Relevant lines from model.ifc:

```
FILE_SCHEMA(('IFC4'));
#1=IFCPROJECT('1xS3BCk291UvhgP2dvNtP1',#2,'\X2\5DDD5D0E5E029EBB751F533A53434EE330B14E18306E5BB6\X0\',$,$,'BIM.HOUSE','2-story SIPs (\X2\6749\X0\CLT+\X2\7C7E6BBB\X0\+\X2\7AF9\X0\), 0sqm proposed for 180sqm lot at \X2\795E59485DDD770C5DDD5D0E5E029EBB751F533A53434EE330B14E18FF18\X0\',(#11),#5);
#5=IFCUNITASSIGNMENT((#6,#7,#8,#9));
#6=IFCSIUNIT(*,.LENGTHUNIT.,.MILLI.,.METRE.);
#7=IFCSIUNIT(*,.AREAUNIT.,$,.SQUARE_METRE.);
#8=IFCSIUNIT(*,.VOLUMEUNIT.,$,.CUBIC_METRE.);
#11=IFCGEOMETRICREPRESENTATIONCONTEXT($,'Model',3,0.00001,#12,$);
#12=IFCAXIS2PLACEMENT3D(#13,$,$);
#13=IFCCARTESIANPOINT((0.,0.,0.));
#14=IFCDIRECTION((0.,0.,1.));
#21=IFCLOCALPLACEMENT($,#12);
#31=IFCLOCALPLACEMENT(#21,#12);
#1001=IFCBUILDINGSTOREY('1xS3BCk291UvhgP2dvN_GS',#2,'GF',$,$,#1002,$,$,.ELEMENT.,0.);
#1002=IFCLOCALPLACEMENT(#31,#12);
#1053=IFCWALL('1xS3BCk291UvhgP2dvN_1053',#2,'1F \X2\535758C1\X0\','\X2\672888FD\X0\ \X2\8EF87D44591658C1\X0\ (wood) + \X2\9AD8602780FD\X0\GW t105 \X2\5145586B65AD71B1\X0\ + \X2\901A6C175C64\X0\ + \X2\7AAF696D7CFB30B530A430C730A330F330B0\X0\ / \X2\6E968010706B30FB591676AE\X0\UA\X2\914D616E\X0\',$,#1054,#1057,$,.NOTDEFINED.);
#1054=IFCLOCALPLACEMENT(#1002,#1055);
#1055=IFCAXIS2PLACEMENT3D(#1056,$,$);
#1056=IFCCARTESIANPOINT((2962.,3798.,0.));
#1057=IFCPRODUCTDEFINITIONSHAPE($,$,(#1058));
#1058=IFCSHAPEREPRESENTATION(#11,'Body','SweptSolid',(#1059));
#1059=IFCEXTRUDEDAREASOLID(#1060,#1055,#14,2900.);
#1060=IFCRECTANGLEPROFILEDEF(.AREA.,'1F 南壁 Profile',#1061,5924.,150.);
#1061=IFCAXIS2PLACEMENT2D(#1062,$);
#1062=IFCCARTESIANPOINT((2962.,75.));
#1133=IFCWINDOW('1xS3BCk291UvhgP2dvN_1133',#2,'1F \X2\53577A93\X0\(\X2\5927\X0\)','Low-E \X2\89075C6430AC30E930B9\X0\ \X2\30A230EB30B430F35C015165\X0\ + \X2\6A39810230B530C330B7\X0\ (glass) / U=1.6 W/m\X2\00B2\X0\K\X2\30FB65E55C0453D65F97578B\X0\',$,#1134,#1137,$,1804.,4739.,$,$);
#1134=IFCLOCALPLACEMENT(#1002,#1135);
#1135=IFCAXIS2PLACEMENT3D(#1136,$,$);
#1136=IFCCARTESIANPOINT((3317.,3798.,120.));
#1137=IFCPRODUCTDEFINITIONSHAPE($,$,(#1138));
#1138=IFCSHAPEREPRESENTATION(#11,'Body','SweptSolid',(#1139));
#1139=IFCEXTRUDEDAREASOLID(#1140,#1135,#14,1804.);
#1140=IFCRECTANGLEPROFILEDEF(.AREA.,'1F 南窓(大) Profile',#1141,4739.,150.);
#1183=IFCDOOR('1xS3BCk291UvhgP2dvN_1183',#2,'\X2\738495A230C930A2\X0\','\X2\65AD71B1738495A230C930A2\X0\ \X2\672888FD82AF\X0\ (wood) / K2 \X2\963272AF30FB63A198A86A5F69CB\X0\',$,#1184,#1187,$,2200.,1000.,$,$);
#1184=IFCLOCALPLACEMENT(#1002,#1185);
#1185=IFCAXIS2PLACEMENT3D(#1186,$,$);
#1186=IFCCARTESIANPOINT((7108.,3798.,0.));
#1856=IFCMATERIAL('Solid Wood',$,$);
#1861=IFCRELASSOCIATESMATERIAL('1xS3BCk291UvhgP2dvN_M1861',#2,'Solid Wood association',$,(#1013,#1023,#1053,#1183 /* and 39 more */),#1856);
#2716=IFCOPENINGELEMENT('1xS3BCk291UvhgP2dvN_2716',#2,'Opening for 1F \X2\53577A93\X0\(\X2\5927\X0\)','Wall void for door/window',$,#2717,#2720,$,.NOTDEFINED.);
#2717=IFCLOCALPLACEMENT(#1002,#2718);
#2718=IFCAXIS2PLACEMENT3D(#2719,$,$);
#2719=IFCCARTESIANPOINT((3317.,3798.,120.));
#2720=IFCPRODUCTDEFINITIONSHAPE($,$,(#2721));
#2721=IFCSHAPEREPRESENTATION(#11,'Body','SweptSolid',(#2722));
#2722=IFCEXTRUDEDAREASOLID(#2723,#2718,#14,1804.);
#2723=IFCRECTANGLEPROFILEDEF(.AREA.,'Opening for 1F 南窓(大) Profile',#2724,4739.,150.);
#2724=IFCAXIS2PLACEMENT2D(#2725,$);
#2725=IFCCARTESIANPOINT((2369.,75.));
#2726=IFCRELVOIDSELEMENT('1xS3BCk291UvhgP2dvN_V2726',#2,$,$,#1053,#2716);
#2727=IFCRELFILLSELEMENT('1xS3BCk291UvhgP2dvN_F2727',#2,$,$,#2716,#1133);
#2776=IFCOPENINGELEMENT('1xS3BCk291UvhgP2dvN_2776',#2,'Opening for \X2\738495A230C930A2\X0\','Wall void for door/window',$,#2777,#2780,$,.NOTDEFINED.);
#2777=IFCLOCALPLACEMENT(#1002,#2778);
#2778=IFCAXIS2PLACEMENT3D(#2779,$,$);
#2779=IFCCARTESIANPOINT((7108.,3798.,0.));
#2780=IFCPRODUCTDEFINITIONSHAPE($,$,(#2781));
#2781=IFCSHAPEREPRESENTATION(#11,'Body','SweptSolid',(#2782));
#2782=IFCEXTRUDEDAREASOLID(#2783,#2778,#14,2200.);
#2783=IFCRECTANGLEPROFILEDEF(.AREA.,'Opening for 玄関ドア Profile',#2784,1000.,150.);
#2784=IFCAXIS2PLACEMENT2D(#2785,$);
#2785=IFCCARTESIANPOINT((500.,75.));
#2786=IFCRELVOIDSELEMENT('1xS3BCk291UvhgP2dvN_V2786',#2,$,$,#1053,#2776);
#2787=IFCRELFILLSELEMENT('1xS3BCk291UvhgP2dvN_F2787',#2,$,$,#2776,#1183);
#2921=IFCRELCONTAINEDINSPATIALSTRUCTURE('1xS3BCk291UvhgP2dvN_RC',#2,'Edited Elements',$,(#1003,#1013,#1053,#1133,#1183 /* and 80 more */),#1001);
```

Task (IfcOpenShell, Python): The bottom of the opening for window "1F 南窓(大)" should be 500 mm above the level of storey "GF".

```python
import numpy as np
import ifcopenshell
import ifcopenshell.api.geometry
import ifcopenshell.geom
import ifcopenshell.util.element
import ifcopenshell.util.placement
import ifcopenshell.util.shape
import ifcopenshell.util.unit

model = ifcopenshell.open("model.ifc")
unit_scale = ifcopenshell.util.unit.calculate_unit_scale(model)

window = model.by_id(1133)
opening = window.FillsVoids[0].RelatingOpeningElement
storey = ifcopenshell.util.element.get_container(window, ifc_class="IfcBuildingStorey")
level = ifcopenshell.util.placement.get_local_placement(storey.ObjectPlacement)[2, 3]

# The opening's origin need not be at the sill, so measure its lowest point.
shape = ifcopenshell.geom.create_shape(ifcopenshell.geom.settings(), opening)
bottom = ifcopenshell.util.shape.get_shape_bottom_elevation(shape, shape.geometry) / unit_scale
dz = level + 500.0 - bottom

shift = np.array([0.0, 0.0, dz])
# The window is not placed relative to its opening, so move both.
for product in (opening, window):
    matrix = ifcopenshell.util.placement.get_local_placement(product.ObjectPlacement)
    matrix[:3, 3] += shift
    ifcopenshell.api.geometry.edit_object_placement(model, product=product, matrix=matrix, is_si=False)

print(f"moved by {dz * unit_scale:+.3f} m")

model.write("model_v2.ifc")
```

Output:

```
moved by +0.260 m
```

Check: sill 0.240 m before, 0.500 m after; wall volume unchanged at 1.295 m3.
